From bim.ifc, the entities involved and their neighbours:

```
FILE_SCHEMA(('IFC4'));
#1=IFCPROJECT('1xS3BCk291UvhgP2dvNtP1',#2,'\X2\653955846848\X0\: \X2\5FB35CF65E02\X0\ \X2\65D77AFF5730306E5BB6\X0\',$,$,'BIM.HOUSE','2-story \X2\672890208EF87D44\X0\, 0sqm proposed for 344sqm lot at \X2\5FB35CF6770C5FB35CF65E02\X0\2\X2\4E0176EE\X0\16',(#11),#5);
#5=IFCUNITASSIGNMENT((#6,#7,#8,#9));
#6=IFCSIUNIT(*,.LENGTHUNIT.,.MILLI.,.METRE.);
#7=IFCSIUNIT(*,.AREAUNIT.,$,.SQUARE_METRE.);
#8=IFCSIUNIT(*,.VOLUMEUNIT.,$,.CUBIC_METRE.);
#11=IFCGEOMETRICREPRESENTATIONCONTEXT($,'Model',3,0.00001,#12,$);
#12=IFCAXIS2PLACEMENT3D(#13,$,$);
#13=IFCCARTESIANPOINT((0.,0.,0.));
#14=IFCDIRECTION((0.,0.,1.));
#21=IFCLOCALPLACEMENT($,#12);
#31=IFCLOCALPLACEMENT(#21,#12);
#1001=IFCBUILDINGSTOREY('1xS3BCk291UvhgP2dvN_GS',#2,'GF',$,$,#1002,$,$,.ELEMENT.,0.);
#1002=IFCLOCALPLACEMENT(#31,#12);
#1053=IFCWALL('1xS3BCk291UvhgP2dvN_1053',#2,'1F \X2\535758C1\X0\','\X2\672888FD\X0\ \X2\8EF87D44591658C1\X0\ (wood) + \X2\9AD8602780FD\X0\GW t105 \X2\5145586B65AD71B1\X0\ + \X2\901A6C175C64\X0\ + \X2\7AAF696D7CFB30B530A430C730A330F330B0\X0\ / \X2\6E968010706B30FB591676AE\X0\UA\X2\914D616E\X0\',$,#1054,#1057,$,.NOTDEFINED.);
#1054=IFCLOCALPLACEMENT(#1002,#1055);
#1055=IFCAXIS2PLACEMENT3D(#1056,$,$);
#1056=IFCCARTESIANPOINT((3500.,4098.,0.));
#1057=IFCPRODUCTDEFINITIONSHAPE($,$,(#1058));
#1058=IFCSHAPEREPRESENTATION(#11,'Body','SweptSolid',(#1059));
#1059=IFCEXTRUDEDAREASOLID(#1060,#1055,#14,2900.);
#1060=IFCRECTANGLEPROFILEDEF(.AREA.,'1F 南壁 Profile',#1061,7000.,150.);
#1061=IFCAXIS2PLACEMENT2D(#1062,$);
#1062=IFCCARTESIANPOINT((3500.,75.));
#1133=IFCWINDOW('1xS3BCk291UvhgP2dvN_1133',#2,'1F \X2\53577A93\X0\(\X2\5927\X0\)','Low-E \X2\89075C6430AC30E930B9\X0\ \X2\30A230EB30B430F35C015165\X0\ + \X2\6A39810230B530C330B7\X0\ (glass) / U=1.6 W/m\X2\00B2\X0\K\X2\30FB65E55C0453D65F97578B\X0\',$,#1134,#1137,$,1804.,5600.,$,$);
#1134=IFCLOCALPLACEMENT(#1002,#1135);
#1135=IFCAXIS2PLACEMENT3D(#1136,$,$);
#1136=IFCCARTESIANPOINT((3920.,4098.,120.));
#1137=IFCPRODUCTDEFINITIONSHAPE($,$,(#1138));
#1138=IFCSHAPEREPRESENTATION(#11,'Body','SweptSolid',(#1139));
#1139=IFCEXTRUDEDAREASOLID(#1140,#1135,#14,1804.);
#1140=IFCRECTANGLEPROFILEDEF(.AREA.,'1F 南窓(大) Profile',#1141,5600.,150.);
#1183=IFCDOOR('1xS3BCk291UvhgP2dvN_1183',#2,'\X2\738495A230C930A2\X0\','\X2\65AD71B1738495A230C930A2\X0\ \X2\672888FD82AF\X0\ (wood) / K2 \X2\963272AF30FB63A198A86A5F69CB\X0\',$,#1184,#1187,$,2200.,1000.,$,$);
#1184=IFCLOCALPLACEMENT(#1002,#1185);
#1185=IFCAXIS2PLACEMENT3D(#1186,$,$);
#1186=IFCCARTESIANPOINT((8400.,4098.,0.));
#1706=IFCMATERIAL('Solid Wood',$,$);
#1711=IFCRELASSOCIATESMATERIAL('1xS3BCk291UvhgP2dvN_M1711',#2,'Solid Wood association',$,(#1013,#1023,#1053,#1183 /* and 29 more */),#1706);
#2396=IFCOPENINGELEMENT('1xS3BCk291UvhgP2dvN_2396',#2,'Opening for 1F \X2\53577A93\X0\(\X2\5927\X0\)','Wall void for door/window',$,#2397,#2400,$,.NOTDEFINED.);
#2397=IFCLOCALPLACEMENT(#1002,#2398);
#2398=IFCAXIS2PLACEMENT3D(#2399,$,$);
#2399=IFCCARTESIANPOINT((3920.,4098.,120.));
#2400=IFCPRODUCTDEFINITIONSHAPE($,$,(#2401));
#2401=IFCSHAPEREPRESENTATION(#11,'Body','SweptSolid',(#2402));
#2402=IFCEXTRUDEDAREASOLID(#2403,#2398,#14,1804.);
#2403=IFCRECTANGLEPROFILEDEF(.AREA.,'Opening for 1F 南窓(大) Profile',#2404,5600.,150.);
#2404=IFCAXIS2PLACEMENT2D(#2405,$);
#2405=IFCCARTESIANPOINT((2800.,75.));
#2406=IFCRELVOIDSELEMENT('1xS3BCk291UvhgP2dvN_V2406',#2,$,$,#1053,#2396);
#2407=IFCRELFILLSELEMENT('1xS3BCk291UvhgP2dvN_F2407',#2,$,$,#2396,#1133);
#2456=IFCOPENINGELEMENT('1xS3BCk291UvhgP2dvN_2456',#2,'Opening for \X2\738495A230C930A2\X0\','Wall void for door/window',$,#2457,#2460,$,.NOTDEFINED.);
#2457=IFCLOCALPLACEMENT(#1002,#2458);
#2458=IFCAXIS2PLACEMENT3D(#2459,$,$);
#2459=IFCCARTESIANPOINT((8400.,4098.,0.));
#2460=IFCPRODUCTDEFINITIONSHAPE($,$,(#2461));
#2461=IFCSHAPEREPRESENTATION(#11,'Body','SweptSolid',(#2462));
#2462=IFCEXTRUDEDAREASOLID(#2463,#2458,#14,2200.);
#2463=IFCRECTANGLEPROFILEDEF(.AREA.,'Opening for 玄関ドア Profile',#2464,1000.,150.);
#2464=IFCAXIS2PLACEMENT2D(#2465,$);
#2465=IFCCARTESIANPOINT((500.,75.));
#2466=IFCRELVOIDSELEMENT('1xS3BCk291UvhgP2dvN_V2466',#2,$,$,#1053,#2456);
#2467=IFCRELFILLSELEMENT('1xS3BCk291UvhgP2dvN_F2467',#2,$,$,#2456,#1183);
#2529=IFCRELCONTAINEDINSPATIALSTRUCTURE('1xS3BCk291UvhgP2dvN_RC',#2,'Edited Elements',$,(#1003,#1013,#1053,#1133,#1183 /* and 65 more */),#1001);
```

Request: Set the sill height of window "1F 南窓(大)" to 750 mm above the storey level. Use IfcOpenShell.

```python
import numpy as np
import ifcopenshell
import ifcopenshell.api.geometry
import ifcopenshell.geom
import ifcopenshell.util.element
import ifcopenshell.util.placement
import ifcopenshell.util.shape
import ifcopenshell.util.unit

model = ifcopenshell.open("bim.ifc")
unit_scale = ifcopenshell.util.unit.calculate_unit_scale(model)

window = model.by_guid("1xS3BCk291UvhgP2dvN_1133")
opening = window.FillsVoids[0].RelatingOpeningElement
storey = ifcopenshell.util.element.get_container(window, ifc_class="IfcBuildingStorey")
level = ifcopenshell.util.placement.get_local_placement(storey.ObjectPlacement)[2, 3]

# The opening's origin need not be at the sill, so measure its lowest point.
shape = ifcopenshell.geom.create_shape(ifcopenshell.geom.settings(), opening)
bottom = ifcopenshell.util.shape.get_shape_bottom_elevation(shape, shape.geometry) / unit_scale
dz = level + 750.0 - bottom

shift = np.array([0.0, 0.0, dz])
# The window is not placed relative to its opening, so move both.
for product in (opening, window):
    matrix = ifcopenshell.util.placement.get_local_placement(product.ObjectPlacement)
    matrix[:3, 3] += shift
    ifcopenshell.api.geometry.edit_object_placement(model, product=product, matrix=matrix, is_si=False)

print(f"moved by {dz * unit_scale:+.3f} m")

model.write("bim_edited.ifc")
```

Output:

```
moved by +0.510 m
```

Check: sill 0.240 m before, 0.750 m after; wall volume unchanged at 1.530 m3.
